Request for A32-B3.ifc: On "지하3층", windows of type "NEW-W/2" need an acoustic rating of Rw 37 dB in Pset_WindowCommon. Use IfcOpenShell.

First a look at what the model holds.

```python
import ifcopenshell
import ifcopenshell.util.element

model = ifcopenshell.open("A32-B3.ifc")
print(model.schema)
storey = next(s for s in model.by_type("IfcBuildingStorey") if s.Name == "지하3층")
windows = [e for e in ifcopenshell.util.element.get_decomposition(storey) if e.is_a("IfcWindow")]
seen = {}
for e in windows:
    element_type = ifcopenshell.util.element.get_type(e)
    key = (element_type.Name if element_type != e and element_type else None, ifcopenshell.util.element.get_pset(e, "Pset_WindowCommon", "AcousticRating"))
    seen[key] = seen.get(key, 0) + 1
for (name, value), count in sorted(seen.items(), key=str):
    print(count, "x", name, "|", value)
```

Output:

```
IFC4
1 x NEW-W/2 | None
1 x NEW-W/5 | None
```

```python
import ifcopenshell
import ifcopenshell.api.pset
import ifcopenshell.util.element

model = ifcopenshell.open("A32-B3.ifc")

storey = next(s for s in model.by_type("IfcBuildingStorey") if s.Name == "지하3층")
windows = [e for e in ifcopenshell.util.element.get_decomposition(storey) if e.is_a("IfcWindow")]

count = 0
for e in windows:
    element_type = ifcopenshell.util.element.get_type(e)
    if element_type in (None, e) or element_type.Name != "NEW-W/2":
        continue
    # add_pset returns the element's existing set when there is one.
    pset = ifcopenshell.api.pset.add_pset(model, product=e, name="Pset_WindowCommon")
    ifcopenshell.api.pset.edit_pset(model, pset=pset, properties={"AcousticRating": "Rw 37 dB"})
    count += 1

print(count, "windows updated")

model.write("A32-B3_edited.ifc")
```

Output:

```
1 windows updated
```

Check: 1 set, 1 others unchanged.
